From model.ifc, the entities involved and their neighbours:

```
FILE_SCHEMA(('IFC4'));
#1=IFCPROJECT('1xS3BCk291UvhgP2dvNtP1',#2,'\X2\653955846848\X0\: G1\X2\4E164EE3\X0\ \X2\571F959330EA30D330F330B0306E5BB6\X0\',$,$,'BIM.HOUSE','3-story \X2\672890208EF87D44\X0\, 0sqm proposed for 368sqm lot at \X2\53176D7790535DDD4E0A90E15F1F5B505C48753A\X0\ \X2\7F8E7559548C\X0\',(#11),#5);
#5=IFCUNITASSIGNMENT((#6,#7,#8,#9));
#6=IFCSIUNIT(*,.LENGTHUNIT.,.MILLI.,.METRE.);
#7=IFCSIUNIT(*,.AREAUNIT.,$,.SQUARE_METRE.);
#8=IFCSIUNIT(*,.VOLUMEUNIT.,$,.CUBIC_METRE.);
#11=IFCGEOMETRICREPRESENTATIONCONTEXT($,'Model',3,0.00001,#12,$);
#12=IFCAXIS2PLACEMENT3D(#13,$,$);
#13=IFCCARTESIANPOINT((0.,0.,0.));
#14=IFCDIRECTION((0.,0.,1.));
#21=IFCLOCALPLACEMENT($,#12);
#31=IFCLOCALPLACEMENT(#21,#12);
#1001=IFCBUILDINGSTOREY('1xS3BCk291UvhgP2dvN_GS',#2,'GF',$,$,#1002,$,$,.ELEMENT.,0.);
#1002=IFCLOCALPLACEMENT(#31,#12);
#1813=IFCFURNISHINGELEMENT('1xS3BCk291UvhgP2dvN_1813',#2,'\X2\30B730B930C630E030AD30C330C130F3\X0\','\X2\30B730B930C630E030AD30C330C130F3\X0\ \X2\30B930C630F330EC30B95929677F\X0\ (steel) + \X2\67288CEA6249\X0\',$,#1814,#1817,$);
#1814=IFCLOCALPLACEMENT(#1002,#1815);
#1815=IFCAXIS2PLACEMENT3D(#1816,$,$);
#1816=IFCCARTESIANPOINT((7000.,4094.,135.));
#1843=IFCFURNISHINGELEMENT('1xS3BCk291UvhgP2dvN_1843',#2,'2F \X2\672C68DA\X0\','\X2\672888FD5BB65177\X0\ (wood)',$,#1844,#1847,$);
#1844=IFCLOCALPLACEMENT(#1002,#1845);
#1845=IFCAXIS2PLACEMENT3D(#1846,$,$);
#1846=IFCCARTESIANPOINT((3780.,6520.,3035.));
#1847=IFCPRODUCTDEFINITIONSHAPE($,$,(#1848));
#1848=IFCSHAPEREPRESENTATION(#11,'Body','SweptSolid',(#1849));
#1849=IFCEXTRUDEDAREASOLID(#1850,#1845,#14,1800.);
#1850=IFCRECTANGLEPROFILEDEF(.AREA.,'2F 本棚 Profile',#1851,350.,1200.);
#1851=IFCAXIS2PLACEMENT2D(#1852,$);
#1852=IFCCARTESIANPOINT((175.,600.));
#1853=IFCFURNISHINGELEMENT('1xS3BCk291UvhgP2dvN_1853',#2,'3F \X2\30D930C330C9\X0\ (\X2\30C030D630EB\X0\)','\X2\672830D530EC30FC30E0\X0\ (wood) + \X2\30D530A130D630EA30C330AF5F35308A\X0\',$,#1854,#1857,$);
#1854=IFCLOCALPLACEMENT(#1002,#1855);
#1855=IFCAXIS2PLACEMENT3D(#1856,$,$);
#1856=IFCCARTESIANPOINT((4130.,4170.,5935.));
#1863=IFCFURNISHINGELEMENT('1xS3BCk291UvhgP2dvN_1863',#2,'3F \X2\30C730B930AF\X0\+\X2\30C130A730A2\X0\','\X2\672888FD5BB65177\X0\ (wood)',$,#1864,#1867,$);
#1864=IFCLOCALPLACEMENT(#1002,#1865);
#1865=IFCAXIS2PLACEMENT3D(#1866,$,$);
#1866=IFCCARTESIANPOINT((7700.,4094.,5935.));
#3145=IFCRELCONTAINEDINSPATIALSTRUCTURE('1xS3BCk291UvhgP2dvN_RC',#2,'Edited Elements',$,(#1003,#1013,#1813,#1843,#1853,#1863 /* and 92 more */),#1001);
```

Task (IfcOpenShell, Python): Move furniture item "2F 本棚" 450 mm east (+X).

```python
import ifcopenshell
import ifcopenshell.api.geometry
import ifcopenshell.util.placement

model = ifcopenshell.open("model.ifc")

item = model.by_guid("1xS3BCk291UvhgP2dvN_1843")
matrix = ifcopenshell.util.placement.get_local_placement(item.ObjectPlacement)
matrix[0, 3] += 450.0
ifcopenshell.api.geometry.edit_object_placement(model, product=item, matrix=matrix, is_si=False)

print(ifcopenshell.util.placement.get_local_placement(item.ObjectPlacement).round(3) + 0.0)

model.write("model_updated.ifc")
```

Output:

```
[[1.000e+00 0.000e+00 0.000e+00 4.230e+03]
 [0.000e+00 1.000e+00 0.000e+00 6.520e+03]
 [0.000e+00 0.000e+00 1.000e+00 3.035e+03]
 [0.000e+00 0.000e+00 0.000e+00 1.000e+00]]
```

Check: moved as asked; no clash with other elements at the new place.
